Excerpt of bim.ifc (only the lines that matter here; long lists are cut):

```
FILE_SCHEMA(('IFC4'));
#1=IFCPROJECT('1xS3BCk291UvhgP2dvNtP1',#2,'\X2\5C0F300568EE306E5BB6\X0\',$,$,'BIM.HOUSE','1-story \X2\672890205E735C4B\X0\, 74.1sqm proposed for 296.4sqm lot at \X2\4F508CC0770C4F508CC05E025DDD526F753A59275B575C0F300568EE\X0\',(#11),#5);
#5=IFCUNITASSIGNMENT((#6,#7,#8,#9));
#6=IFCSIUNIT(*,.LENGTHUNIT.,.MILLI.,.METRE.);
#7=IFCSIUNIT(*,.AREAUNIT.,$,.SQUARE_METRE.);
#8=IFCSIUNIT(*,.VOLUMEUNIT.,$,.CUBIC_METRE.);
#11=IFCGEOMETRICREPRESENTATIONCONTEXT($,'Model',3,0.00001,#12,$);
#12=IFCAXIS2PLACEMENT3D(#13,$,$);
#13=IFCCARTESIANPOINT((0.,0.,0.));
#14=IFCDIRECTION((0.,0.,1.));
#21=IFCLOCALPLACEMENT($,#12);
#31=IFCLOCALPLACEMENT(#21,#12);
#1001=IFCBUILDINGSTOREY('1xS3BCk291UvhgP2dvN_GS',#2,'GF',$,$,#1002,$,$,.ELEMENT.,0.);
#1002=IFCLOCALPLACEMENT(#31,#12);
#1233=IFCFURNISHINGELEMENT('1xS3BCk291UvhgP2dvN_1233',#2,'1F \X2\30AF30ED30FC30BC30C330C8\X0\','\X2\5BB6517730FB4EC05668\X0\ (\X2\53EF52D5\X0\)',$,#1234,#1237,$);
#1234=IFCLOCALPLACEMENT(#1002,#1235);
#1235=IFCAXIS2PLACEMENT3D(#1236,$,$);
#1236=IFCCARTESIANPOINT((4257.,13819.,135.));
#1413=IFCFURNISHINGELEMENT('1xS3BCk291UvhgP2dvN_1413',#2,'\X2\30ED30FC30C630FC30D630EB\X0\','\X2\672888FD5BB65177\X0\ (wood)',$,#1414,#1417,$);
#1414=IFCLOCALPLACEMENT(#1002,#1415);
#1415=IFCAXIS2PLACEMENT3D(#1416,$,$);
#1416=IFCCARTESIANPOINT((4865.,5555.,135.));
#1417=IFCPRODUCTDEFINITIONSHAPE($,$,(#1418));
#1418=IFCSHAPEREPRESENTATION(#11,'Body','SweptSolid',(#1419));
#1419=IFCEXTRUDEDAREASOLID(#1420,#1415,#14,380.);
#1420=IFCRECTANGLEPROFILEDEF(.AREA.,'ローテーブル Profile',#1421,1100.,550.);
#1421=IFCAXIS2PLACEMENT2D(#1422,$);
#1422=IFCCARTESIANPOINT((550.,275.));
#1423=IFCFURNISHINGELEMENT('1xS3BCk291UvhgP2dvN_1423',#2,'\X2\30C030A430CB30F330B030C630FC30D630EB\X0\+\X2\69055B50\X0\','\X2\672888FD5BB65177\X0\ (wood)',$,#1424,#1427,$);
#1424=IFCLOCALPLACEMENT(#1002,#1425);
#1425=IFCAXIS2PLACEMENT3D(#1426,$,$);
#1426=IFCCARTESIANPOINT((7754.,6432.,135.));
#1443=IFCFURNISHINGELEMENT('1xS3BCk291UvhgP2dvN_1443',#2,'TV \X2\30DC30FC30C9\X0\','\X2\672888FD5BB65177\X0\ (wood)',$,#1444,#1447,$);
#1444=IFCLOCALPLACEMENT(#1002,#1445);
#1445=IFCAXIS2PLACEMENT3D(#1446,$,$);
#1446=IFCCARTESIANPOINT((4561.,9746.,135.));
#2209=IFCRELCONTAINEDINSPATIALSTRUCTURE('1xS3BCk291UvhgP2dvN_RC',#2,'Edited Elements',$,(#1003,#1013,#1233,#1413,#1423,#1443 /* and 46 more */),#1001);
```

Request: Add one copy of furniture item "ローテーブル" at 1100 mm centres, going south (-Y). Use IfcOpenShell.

```python
import numpy as np
import ifcopenshell
import ifcopenshell.api.geometry
import ifcopenshell.api.root
import ifcopenshell.util.element
import ifcopenshell.util.placement
import ifcopenshell.util.unit

model = ifcopenshell.open("bim.ifc")
unit_scale = ifcopenshell.util.unit.calculate_unit_scale(model)


def reuse_history(source, copy):
    """copy_class also copies each property set's owner history, people and application; keep the originals."""
    for rel in copy.IsDefinedBy:
        if rel.is_a("IfcRelDefinesByProperties") and (history := rel.RelatingPropertyDefinition.OwnerHistory):
            rel.RelatingPropertyDefinition.OwnerHistory = source.OwnerHistory
            ifcopenshell.util.element.remove_deep2(model, history)


source = model.by_guid("1xS3BCk291UvhgP2dvN_1413")
base = ifcopenshell.util.placement.get_local_placement(source.ObjectPlacement)
step = np.array([0.0, -1.0, 0.0]) * 1.1 / unit_scale

for i in range(1, 2):
    copy = ifcopenshell.api.root.copy_class(model, product=source)
    copy.Representation = ifcopenshell.util.element.copy_deep(
        model, source.Representation, exclude=["IfcGeometricRepresentationContext", "IfcRepresentationMap"]
    )
    reuse_history(source, copy)
    matrix = base.copy()
    matrix[:3, 3] += i * step
    print("added at", matrix[:3, 3].round(3) + 0.0)
    ifcopenshell.api.geometry.edit_object_placement(model, product=copy, matrix=matrix, is_si=False)

model.write("bim_rev.ifc")
```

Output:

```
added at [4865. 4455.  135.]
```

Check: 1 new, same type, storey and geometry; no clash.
